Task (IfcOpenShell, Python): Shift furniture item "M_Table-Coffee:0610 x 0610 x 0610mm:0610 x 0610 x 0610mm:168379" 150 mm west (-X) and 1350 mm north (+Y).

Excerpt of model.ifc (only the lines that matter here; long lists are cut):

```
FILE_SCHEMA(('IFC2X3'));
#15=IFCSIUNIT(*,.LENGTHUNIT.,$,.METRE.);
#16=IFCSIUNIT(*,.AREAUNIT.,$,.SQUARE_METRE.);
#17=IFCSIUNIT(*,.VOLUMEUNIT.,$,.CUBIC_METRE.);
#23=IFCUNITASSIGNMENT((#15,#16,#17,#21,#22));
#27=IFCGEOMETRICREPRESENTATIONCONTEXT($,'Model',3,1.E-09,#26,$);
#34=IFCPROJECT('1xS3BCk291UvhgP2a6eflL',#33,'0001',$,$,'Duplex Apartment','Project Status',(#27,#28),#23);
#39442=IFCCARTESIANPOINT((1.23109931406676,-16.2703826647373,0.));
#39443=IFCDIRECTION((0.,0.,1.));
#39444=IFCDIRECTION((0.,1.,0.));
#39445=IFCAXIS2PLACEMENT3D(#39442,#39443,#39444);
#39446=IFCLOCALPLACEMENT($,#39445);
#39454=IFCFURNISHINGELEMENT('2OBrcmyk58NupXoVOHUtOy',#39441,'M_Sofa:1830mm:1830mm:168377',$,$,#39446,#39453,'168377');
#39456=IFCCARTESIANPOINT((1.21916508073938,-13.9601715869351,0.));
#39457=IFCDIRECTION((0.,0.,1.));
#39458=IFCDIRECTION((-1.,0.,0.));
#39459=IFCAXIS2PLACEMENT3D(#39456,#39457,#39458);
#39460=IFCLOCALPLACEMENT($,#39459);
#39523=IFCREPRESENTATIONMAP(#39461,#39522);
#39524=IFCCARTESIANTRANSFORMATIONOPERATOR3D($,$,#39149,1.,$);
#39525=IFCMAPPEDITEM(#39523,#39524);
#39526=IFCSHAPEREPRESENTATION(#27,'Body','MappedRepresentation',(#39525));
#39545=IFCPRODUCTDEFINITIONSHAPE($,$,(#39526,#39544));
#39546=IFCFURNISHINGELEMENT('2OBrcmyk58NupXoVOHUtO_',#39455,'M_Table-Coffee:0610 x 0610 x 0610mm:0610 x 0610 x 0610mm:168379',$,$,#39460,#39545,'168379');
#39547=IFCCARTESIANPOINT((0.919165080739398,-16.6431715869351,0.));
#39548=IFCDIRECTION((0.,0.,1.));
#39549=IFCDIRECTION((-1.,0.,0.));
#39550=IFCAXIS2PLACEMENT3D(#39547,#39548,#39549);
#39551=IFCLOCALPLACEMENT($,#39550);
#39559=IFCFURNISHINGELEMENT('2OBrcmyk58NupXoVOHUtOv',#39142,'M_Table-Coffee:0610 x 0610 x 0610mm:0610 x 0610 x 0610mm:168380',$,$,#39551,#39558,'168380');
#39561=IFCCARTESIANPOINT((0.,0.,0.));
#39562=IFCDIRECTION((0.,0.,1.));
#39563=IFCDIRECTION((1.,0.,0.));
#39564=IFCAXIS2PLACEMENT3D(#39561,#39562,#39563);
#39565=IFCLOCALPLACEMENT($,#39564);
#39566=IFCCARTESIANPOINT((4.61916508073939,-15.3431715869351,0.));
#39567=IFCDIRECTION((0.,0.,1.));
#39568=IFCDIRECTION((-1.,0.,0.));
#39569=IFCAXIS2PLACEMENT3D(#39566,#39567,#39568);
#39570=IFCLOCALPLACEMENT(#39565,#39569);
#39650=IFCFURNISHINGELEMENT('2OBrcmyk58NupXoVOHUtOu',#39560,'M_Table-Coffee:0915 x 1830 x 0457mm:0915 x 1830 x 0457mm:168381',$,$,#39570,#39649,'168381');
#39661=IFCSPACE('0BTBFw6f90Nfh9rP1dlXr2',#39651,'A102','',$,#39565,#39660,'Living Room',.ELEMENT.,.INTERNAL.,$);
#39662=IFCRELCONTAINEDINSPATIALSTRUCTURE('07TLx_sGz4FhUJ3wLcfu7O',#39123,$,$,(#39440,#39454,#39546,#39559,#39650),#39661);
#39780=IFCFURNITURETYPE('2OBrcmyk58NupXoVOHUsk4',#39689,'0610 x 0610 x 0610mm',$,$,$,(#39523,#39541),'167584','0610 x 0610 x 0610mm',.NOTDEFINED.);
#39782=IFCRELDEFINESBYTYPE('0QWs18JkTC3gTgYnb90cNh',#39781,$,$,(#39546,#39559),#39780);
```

```python
import ifcopenshell
import ifcopenshell.api.geometry
import ifcopenshell.util.placement

model = ifcopenshell.open("model.ifc")

item = model.by_id(39546)
matrix = ifcopenshell.util.placement.get_local_placement(item.ObjectPlacement)
matrix[0, 3] -= 0.15
matrix[1, 3] += 1.35
ifcopenshell.api.geometry.edit_object_placement(model, product=item, matrix=matrix, is_si=False)

print(ifcopenshell.util.placement.get_local_placement(item.ObjectPlacement).round(3) + 0.0)

model.write("model_updated.ifc")
```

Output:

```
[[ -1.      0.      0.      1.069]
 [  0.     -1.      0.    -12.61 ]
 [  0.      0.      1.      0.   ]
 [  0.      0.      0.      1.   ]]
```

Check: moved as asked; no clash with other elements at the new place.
